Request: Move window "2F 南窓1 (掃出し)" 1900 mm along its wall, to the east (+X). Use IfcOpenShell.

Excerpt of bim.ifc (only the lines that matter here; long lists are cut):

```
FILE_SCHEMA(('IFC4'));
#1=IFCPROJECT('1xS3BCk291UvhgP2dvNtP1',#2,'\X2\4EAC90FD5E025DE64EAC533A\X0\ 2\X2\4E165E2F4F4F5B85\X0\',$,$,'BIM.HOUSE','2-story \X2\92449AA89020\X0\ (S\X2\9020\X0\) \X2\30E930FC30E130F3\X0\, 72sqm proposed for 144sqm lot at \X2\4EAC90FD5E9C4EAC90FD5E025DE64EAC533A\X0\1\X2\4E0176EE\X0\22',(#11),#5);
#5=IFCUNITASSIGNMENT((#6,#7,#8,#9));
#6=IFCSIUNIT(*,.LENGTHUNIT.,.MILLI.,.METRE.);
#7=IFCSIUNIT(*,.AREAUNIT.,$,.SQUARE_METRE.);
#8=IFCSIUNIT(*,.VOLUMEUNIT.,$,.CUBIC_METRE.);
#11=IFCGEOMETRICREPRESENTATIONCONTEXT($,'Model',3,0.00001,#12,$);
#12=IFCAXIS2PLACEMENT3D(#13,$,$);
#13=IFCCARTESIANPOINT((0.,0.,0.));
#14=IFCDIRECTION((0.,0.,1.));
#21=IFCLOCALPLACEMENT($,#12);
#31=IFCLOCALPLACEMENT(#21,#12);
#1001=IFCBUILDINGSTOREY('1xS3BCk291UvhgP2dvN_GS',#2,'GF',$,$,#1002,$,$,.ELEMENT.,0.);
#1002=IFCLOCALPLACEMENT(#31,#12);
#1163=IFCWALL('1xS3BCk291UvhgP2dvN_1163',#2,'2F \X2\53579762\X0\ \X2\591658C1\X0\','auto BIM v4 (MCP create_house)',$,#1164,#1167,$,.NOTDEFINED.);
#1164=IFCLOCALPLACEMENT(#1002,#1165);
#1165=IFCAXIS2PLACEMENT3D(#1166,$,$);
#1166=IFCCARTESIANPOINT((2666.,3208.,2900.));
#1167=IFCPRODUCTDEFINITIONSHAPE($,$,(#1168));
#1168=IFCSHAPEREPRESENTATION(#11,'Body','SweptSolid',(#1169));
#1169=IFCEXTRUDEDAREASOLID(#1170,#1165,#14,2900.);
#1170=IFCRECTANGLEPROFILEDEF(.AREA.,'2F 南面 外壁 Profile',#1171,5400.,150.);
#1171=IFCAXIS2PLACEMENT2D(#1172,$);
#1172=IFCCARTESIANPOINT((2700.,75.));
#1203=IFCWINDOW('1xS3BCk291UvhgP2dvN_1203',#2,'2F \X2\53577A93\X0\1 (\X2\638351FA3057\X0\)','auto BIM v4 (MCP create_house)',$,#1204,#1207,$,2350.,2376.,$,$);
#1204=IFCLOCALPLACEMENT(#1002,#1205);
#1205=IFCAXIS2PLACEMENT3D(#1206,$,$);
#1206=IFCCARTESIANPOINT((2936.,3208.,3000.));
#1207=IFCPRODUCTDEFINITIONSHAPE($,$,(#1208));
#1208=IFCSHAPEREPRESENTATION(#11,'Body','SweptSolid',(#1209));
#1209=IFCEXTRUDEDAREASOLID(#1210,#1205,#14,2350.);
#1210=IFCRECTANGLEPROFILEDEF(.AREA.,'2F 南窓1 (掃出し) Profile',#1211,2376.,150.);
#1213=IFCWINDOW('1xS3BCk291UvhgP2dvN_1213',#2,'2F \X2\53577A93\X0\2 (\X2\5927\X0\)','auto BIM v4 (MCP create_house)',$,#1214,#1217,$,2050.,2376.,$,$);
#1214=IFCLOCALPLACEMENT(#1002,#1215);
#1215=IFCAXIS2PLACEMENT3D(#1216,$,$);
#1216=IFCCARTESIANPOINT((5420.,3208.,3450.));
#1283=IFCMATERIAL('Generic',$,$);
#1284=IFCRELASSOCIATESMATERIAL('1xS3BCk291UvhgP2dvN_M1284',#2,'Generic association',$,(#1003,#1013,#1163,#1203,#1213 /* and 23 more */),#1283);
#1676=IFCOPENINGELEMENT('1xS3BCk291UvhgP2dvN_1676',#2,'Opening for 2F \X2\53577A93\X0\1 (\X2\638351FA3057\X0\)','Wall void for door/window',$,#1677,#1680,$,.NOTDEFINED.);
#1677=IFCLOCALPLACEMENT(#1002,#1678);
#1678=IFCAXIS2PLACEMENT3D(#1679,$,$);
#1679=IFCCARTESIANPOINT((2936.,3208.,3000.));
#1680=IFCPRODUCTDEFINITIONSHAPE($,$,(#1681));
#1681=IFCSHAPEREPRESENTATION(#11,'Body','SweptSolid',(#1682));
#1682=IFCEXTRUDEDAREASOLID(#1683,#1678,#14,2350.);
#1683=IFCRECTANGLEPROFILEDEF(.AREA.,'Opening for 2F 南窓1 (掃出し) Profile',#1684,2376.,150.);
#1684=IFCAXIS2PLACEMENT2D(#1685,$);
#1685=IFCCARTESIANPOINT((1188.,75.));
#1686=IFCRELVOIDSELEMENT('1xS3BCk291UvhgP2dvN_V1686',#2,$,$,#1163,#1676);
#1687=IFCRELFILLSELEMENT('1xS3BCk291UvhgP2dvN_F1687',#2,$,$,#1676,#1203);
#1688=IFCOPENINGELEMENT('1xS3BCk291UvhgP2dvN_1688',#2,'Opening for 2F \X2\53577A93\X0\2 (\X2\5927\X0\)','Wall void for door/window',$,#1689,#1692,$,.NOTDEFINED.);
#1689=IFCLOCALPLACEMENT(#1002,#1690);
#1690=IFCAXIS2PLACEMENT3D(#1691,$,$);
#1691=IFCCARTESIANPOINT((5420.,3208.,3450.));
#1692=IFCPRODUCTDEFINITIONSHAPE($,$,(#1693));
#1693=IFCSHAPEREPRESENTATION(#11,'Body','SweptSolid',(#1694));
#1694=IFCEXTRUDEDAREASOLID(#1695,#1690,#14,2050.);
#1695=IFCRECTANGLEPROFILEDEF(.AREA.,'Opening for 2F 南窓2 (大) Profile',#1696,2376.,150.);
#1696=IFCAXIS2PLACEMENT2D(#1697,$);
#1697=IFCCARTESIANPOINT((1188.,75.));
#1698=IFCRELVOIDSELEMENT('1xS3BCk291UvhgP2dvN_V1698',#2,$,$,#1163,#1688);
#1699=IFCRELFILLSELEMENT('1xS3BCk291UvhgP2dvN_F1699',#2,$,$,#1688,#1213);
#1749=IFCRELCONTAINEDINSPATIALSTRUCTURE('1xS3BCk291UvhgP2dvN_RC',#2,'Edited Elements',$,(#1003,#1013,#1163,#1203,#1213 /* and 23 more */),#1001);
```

```python
import ifcopenshell
import ifcopenshell.api.geometry
import ifcopenshell.util.placement
import ifcopenshell.util.unit

model = ifcopenshell.open("bim.ifc")
unit_scale = ifcopenshell.util.unit.calculate_unit_scale(model)

window = model.by_guid("1xS3BCk291UvhgP2dvN_1203")
opening = window.FillsVoids[0].RelatingOpeningElement
wall = opening.VoidsElements[0].RelatingBuildingElement

wall_matrix = ifcopenshell.util.placement.get_local_placement(wall.ObjectPlacement)
shift = wall_matrix[:3, 0] * 1.9 / unit_scale
before = ifcopenshell.util.placement.get_local_placement(window.ObjectPlacement)[:3, 3].copy()

# The window is not placed relative to its opening, so move both.
for product in (opening, window):
    matrix = ifcopenshell.util.placement.get_local_placement(product.ObjectPlacement)
    matrix[:3, 3] += shift
    ifcopenshell.api.geometry.edit_object_placement(model, product=product, matrix=matrix, is_si=False)

after = ifcopenshell.util.placement.get_local_placement(window.ObjectPlacement)[:3, 3]
print("window moved by", (after - before).round(3) + 0.0)

model.write("bim-out.ifc")
```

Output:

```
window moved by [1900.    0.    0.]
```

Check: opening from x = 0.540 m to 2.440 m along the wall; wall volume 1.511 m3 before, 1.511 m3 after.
